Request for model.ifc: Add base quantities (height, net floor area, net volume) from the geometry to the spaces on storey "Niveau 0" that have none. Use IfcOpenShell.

First a look at what the model holds.

```python
import ifcopenshell
import ifcopenshell.util.element
import ifcopenshell.util.unit

model = ifcopenshell.open("model.ifc")
print(model.schema)
for unit_type in ("LENGTHUNIT", "AREAUNIT", "VOLUMEUNIT"):
    print(unit_type, ifcopenshell.util.unit.calculate_unit_scale(model, unit_type))
storey = next(s for s in model.by_type("IfcBuildingStorey") if s.Name == "Niveau 0")
spaces = [e for e in ifcopenshell.util.element.get_decomposition(storey) if e.is_a("IfcSpace")]
for e in sorted(spaces, key=lambda e: e.id()):
    print(e.id(), e.is_a(), e.Name, list(ifcopenshell.util.element.get_psets(e, qtos_only=True)), sep=" | ")
```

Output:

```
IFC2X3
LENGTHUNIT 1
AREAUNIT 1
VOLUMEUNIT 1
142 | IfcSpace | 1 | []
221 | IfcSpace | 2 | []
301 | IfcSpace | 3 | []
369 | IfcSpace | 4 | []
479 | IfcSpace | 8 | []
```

```python
import ifcopenshell
import ifcopenshell.api.pset
import ifcopenshell.geom
import ifcopenshell.util.element
import ifcopenshell.util.shape
import ifcopenshell.util.unit

model = ifcopenshell.open("model.ifc")
unit_scale = ifcopenshell.util.unit.calculate_unit_scale(model)
area_scale = ifcopenshell.util.unit.calculate_unit_scale(model, "AREAUNIT")
volume_scale = ifcopenshell.util.unit.calculate_unit_scale(model, "VOLUMEUNIT")
settings = ifcopenshell.geom.settings()

storey = next(s for s in model.by_type("IfcBuildingStorey") if s.Name == "Niveau 0")
spaces = [e for e in ifcopenshell.util.element.get_decomposition(storey) if e.is_a("IfcSpace")]

for e in sorted(spaces, key=lambda e: e.id()):
    if ifcopenshell.util.element.get_psets(e, qtos_only=True, should_inherit=False):
        continue
    # Geometry comes back in metres, in the element's own axes.
    shape = ifcopenshell.geom.create_shape(settings, e)
    values = {
        "Height": ifcopenshell.util.shape.get_z(shape.geometry) / unit_scale,
        "NetFloorArea": ifcopenshell.util.shape.get_footprint_area(shape.geometry) / area_scale,
        "NetVolume": ifcopenshell.util.shape.get_volume(shape.geometry) / volume_scale,
    }
    qto = ifcopenshell.api.pset.add_qto(model, product=e, name="BaseQuantities")
    ifcopenshell.api.pset.edit_qto(model, qto=qto, properties=values)
    print(e.id(), {k: round(v, 3) for k, v in values.items()})

model.write("model_edited.ifc")
```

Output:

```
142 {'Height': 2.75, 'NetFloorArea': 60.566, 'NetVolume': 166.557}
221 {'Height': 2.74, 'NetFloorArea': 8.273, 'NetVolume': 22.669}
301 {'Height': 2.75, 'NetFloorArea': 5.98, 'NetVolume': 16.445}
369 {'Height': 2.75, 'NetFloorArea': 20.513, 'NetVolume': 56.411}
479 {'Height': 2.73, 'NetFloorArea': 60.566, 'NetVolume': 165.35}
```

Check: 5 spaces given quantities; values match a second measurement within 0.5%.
